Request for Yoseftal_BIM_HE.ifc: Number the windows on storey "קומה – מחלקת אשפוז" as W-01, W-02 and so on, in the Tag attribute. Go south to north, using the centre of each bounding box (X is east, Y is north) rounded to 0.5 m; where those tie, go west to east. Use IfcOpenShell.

First a look at what the model holds.

```python
import ifcopenshell
import ifcopenshell.util.element
import ifcopenshell.util.placement

model = ifcopenshell.open("Yoseftal_BIM_HE.ifc")
print(model.schema)
storey = next(s for s in model.by_type("IfcBuildingStorey") if s.Name == "קומה – מחלקת אשפוז")
windows = [e for e in ifcopenshell.util.element.get_decomposition(storey) if e.is_a("IfcWindow")]
for e in sorted(windows, key=lambda e: e.id()):
    origin = ifcopenshell.util.placement.get_local_placement(e.ObjectPlacement)[:3, 3]
    print(e.id(), e.Tag, e.Name, origin.round(2) + 0.0, sep=" | ")
```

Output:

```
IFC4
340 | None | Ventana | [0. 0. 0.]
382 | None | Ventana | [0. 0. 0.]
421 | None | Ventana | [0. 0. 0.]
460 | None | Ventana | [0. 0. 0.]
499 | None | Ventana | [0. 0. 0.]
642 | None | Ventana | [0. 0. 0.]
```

```python
import ifcopenshell
import ifcopenshell.geom
import ifcopenshell.util.element
import ifcopenshell.util.shape

model = ifcopenshell.open("Yoseftal_BIM_HE.ifc")
settings = ifcopenshell.geom.settings()
settings.set("use-world-coords", True)


def centre(element):
    shape = ifcopenshell.geom.create_shape(settings, element)
    return ifcopenshell.util.shape.get_bbox_centroid(shape.geometry)


storey = next(s for s in model.by_type("IfcBuildingStorey") if s.Name == "קומה – מחלקת אשפוז")
windows = [e for e in ifcopenshell.util.element.get_decomposition(storey) if e.is_a("IfcWindow")]

# Insertion points can sit at a corner or the storey origin, so sort by the geometry (in metres).
centres = {e: centre(e) for e in windows}
windows.sort(key=lambda e: (round(centres[e][1] / 0.5), centres[e][0]))

for i, e in enumerate(windows, start=1):
    number = f"W-{i:02d}"
    e.Tag = number
    print(e.id(), number)

model.write("Yoseftal_BIM_HE_v2.ifc")
```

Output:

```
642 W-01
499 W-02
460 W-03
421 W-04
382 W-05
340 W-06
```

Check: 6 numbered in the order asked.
